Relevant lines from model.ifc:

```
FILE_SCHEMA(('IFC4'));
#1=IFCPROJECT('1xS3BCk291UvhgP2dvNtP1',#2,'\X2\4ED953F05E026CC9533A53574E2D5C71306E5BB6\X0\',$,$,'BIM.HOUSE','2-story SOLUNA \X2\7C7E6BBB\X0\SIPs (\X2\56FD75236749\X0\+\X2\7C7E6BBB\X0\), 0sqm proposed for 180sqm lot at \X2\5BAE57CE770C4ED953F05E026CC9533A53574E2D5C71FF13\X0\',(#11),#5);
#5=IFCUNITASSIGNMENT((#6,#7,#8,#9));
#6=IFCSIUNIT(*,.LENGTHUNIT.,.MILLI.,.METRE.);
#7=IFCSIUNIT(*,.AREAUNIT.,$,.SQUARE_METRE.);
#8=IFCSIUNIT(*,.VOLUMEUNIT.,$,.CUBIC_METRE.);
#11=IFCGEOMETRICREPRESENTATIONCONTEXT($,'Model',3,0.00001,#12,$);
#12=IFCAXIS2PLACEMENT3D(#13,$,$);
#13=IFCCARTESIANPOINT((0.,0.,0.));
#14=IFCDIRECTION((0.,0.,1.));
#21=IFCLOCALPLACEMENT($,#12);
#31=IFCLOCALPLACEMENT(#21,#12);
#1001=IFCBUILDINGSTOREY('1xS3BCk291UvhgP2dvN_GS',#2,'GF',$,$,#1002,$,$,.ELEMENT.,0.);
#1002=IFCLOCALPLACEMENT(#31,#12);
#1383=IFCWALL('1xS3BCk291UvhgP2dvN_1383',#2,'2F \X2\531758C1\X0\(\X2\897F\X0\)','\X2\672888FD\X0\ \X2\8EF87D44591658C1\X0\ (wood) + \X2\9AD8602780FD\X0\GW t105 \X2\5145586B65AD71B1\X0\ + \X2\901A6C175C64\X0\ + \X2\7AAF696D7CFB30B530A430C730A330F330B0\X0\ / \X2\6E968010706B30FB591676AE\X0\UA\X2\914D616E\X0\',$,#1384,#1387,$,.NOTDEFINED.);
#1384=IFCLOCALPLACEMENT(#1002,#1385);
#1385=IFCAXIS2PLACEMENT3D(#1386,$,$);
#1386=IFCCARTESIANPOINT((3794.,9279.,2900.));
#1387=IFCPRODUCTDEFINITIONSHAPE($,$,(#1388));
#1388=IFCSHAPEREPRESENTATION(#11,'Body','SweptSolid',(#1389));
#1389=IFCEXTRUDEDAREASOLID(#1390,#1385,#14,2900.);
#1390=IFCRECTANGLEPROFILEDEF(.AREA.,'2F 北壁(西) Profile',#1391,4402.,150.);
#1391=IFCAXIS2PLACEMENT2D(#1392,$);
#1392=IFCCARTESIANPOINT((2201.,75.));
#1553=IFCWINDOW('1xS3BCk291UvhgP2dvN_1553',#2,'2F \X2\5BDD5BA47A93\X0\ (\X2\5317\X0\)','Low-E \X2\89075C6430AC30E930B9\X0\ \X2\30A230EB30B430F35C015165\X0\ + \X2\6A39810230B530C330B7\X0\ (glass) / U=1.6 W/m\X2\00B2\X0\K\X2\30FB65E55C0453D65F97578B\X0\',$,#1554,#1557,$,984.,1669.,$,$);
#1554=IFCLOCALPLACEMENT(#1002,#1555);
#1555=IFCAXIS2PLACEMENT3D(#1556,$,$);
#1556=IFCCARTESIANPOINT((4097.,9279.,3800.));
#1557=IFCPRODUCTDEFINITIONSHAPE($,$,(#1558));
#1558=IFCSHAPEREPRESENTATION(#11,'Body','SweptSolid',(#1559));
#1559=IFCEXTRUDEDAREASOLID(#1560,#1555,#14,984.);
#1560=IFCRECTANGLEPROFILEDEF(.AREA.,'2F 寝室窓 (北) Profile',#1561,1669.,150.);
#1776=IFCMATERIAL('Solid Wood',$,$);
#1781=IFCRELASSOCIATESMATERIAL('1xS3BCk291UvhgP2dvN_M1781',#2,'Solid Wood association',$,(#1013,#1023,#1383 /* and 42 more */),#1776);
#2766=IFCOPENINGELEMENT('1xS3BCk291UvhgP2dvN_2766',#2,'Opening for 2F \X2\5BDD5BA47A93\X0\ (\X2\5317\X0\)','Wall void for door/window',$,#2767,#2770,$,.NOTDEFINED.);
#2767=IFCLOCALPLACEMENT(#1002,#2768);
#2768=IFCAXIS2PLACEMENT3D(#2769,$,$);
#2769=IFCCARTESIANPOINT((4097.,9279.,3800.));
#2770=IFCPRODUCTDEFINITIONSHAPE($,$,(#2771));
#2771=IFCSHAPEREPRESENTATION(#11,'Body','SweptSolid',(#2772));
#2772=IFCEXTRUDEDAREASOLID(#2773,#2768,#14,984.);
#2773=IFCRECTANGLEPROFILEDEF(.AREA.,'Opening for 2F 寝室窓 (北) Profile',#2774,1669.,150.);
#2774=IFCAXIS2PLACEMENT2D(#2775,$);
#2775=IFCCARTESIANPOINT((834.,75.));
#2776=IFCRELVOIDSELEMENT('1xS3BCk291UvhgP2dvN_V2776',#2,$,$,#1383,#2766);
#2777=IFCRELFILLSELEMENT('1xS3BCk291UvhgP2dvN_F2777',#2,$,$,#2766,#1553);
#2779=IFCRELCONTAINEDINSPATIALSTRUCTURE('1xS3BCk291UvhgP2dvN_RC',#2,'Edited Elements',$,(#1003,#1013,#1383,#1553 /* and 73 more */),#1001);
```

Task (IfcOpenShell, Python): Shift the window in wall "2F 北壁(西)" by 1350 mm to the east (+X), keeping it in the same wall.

```python
import ifcopenshell
import ifcopenshell.api.geometry
import ifcopenshell.util.placement

model = ifcopenshell.open("model.ifc")

window = model.by_guid("1xS3BCk291UvhgP2dvN_1553")
opening = window.FillsVoids[0].RelatingOpeningElement
wall = opening.VoidsElements[0].RelatingBuildingElement

wall_matrix = ifcopenshell.util.placement.get_local_placement(wall.ObjectPlacement)
shift = wall_matrix[:3, 0] * 1350.0
before = ifcopenshell.util.placement.get_local_placement(window.ObjectPlacement)[:3, 3].copy()

# The window is not placed relative to its opening, so move both.
for product in (opening, window):
    matrix = ifcopenshell.util.placement.get_local_placement(product.ObjectPlacement)
    matrix[:3, 3] += shift
    ifcopenshell.api.geometry.edit_object_placement(model, product=product, matrix=matrix, is_si=False)

after = ifcopenshell.util.placement.get_local_placement(window.ObjectPlacement)[:3, 3]
print("window moved by", (after - before).round(3) + 0.0)

model.write("model-out.ifc")
```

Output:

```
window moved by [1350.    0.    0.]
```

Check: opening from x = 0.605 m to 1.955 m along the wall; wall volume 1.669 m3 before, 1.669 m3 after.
